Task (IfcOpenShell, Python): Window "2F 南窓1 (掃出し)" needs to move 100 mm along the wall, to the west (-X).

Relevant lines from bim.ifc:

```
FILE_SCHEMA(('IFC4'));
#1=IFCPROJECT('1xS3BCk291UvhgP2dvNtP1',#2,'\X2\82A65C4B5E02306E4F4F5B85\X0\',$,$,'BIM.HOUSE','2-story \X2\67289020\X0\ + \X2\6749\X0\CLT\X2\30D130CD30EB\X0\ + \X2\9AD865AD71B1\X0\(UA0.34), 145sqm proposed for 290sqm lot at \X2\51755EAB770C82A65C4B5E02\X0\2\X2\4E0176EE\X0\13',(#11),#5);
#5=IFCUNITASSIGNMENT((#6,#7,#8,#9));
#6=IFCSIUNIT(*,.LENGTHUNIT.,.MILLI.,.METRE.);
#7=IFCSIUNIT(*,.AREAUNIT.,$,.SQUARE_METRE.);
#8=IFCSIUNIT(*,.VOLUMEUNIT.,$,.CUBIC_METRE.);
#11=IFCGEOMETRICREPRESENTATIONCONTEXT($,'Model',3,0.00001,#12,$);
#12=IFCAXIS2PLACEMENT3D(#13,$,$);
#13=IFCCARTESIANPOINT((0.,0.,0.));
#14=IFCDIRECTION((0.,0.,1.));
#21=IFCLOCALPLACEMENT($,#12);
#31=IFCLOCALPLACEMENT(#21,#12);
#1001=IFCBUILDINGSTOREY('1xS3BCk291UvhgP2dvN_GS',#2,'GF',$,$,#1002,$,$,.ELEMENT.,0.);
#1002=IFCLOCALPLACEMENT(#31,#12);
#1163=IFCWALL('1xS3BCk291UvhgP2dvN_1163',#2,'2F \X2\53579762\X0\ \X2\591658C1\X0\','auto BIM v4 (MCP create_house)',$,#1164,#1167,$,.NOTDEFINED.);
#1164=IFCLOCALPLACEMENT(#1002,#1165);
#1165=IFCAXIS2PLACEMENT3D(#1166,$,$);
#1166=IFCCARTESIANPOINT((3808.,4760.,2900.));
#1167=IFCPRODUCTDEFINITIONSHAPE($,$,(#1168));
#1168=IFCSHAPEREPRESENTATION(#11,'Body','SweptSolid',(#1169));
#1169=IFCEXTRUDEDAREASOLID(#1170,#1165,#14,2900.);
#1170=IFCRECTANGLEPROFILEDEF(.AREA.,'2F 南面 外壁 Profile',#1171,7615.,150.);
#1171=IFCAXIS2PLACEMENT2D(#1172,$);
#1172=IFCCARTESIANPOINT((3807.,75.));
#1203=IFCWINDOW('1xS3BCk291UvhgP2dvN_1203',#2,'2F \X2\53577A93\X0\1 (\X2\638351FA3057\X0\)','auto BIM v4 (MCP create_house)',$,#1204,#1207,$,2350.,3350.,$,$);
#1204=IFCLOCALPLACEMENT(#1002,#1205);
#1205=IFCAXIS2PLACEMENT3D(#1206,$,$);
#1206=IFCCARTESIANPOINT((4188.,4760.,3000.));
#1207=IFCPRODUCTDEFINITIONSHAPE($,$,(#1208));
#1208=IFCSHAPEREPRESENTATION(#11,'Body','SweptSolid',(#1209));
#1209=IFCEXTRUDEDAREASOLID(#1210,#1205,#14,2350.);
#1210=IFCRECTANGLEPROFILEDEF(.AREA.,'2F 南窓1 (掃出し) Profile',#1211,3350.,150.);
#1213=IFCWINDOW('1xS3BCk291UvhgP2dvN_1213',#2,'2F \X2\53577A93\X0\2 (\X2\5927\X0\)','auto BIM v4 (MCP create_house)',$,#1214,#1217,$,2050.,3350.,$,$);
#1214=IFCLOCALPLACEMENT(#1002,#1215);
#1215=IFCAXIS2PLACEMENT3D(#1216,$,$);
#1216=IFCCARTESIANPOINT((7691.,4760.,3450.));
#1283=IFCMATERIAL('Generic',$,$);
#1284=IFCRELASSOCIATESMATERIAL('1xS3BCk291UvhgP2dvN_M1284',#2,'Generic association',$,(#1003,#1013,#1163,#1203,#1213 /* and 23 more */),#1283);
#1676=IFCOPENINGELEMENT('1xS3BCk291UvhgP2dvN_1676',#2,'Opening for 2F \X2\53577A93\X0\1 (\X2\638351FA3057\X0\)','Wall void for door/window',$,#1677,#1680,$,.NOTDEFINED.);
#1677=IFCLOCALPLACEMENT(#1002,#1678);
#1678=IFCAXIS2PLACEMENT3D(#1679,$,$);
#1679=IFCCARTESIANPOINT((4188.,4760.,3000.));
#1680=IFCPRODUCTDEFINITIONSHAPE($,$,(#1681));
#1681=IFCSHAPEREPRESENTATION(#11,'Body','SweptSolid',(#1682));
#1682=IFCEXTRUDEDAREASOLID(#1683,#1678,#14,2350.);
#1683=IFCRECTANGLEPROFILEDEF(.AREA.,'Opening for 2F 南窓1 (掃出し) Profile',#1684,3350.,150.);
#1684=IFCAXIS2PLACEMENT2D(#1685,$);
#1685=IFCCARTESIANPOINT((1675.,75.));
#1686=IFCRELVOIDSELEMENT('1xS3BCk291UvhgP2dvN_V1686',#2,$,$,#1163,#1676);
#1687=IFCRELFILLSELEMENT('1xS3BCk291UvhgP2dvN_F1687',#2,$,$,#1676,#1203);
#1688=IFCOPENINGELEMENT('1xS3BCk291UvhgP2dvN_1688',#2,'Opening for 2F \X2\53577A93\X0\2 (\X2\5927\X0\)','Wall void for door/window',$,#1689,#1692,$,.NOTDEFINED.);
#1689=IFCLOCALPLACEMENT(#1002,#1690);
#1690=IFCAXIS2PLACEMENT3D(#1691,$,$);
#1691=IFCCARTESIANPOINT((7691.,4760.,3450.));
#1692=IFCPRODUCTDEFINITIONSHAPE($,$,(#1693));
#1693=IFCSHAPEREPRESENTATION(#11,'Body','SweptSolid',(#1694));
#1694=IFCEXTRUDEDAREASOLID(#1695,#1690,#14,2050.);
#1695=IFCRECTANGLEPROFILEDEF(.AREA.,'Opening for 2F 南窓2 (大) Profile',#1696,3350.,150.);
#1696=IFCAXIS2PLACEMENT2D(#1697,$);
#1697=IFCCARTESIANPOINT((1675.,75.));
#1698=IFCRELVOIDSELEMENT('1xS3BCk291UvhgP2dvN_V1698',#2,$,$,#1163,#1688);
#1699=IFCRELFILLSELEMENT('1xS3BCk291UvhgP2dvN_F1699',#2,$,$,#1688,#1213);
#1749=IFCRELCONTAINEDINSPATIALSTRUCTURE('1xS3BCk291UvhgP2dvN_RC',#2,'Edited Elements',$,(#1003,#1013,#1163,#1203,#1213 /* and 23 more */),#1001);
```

```python
import ifcopenshell
import ifcopenshell.api.geometry
import ifcopenshell.util.placement

model = ifcopenshell.open("bim.ifc")

window = model.by_guid("1xS3BCk291UvhgP2dvN_1203")
opening = window.FillsVoids[0].RelatingOpeningElement
wall = opening.VoidsElements[0].RelatingBuildingElement

wall_matrix = ifcopenshell.util.placement.get_local_placement(wall.ObjectPlacement)
shift = wall_matrix[:3, 0] * -100.0
before = ifcopenshell.util.placement.get_local_placement(window.ObjectPlacement)[:3, 3].copy()

# The window is not placed relative to its opening, so move both.
for product in (opening, window):
    matrix = ifcopenshell.util.placement.get_local_placement(product.ObjectPlacement)
    matrix[:3, 3] += shift
    ifcopenshell.api.geometry.edit_object_placement(model, product=product, matrix=matrix, is_si=False)

after = ifcopenshell.util.placement.get_local_placement(window.ObjectPlacement)[:3, 3]
print("window moved by", (after - before).round(3) + 0.0)

model.write("bim-out.ifc")
```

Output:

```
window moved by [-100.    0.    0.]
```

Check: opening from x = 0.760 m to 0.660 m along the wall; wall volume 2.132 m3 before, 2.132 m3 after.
